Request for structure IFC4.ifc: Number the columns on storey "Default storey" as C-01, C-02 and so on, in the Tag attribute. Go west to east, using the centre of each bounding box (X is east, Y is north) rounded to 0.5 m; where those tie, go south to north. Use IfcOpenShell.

First a look at what the model holds.

```python
import ifcopenshell
import ifcopenshell.util.element
import ifcopenshell.util.placement

model = ifcopenshell.open("structure IFC4.ifc")
print(model.schema)
storey = next(s for s in model.by_type("IfcBuildingStorey") if s.Name == "Default storey")
columns = [e for e in ifcopenshell.util.element.get_decomposition(storey) if e.is_a("IfcColumn")]
for e in sorted(columns, key=lambda e: e.id()):
    origin = ifcopenshell.util.placement.get_local_placement(e.ObjectPlacement)[:3, 3]
    print(e.id(), e.Tag, e.Name, origin.round(2) + 0.0, sep=" | ")
```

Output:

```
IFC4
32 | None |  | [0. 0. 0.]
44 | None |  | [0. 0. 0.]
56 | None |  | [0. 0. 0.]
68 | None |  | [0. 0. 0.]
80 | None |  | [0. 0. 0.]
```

```python
import ifcopenshell
import ifcopenshell.geom
import ifcopenshell.util.element
import ifcopenshell.util.shape

model = ifcopenshell.open("structure IFC4.ifc")
settings = ifcopenshell.geom.settings()
settings.set("use-world-coords", True)


def centre(element):
    shape = ifcopenshell.geom.create_shape(settings, element)
    return ifcopenshell.util.shape.get_bbox_centroid(shape.geometry)


storey = next(s for s in model.by_type("IfcBuildingStorey") if s.Name == "Default storey")
columns = [e for e in ifcopenshell.util.element.get_decomposition(storey) if e.is_a("IfcColumn")]

# Insertion points can sit at a corner or the storey origin, so sort by the geometry (in metres).
centres = {e: centre(e) for e in columns}
columns.sort(key=lambda e: (round(centres[e][0] / 0.5), centres[e][1]))

for i, e in enumerate(columns, start=1):
    number = f"C-{i:02d}"
    e.Tag = number
    print(e.id(), number)

model.write("structure IFC4_edited.ifc")
```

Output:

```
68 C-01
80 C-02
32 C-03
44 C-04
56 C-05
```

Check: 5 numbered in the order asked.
